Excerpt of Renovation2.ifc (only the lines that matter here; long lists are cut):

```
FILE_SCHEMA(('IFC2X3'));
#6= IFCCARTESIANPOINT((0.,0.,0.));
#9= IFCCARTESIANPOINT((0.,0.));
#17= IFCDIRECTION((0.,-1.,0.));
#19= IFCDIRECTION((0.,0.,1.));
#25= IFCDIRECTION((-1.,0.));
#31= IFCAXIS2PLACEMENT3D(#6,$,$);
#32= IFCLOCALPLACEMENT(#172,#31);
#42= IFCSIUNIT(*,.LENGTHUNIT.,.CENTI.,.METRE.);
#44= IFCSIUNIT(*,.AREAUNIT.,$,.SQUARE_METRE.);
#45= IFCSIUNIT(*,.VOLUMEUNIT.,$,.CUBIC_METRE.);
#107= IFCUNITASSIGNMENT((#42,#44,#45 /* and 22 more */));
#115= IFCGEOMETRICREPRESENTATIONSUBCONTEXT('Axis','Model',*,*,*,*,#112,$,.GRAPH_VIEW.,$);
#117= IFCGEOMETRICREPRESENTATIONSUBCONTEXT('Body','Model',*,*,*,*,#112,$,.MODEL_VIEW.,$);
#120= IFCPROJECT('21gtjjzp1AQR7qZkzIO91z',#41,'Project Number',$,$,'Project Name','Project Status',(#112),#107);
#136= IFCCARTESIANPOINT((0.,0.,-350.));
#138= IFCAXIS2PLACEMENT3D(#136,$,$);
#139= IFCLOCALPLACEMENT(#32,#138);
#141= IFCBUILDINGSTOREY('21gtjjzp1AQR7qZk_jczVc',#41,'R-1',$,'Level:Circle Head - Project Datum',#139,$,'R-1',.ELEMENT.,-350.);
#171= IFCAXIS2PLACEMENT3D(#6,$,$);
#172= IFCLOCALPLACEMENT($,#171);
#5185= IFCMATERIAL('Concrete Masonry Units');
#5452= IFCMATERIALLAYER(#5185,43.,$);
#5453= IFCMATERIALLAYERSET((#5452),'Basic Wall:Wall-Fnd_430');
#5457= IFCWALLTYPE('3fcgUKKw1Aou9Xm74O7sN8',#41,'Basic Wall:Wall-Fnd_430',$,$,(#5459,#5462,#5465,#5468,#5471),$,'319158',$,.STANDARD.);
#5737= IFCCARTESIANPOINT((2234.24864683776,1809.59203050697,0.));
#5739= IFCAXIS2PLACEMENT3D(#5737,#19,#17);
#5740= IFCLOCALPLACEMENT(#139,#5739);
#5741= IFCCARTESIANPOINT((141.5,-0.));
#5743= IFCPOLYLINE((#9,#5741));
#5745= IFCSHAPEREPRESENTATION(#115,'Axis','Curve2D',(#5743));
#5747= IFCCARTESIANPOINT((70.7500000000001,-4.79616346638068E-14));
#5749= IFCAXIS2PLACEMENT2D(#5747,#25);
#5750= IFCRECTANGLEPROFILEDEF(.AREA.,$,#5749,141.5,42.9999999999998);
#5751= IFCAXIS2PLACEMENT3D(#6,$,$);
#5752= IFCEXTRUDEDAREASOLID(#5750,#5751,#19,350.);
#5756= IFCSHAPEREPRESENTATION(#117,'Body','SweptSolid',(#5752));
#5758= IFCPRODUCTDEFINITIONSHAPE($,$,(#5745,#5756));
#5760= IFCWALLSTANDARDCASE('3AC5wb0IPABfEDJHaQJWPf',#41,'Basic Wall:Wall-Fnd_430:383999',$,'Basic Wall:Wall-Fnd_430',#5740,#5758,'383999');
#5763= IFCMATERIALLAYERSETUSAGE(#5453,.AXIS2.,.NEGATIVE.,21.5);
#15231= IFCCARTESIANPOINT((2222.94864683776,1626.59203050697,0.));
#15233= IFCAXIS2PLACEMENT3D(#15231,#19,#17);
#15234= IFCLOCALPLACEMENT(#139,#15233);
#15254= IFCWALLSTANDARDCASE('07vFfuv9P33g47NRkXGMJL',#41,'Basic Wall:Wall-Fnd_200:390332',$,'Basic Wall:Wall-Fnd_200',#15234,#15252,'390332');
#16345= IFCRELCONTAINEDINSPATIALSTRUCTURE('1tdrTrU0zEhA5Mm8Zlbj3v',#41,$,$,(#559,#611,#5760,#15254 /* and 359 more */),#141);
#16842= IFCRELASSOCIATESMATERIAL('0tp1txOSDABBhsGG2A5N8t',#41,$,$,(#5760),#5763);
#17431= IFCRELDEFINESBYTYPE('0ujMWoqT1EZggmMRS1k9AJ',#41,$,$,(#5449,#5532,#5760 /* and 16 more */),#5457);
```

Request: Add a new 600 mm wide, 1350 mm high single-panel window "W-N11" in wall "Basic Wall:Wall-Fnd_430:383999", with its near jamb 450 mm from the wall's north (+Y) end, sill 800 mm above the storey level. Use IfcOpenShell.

```python
import numpy as np
import ifcopenshell
import ifcopenshell.api.feature
import ifcopenshell.api.geometry
import ifcopenshell.api.root
import ifcopenshell.api.spatial
import ifcopenshell.api.type
import ifcopenshell.geom
import ifcopenshell.util.element
import ifcopenshell.util.placement
import ifcopenshell.util.representation
import ifcopenshell.util.shape
import ifcopenshell.util.unit

model = ifcopenshell.open("Renovation2.ifc")
unit_scale = ifcopenshell.util.unit.calculate_unit_scale(model)
settings = ifcopenshell.geom.settings()


def volume(element):
    """Net volume in cubic metres, openings subtracted."""
    shape = ifcopenshell.geom.create_shape(settings, element)
    return ifcopenshell.util.shape.get_volume(shape.geometry)


wall = model.by_guid("3AC5wb0IPABfEDJHaQJWPf")
storey = ifcopenshell.util.element.get_container(wall, ifc_class="IfcBuildingStorey")
context = ifcopenshell.util.representation.get_context(model, "Model", "Body", "MODEL_VIEW")
before = volume(wall)

width, height, from_end, sill = 0.6, 1.35, 0.45, 0.8  # metres

# The wall runs along its own X axis, and the end named is its -X end.
wall_shape = ifcopenshell.geom.create_shape(settings, wall)
x, y, z = ifcopenshell.util.shape.get_vertices(wall_shape.geometry).T
start = x.min() + from_end
face, thickness = float(y.min()), float(y.max() - y.min())
wall_matrix = ifcopenshell.util.placement.get_local_placement(wall.ObjectPlacement)
level = ifcopenshell.util.placement.get_local_placement(storey.ObjectPlacement)[2, 3]


def in_wall(x, y):
    """Placement at x, y metres in the wall's axes, at sill height."""
    matrix = wall_matrix.copy()
    matrix[:, 3] = wall_matrix @ np.array([x / unit_scale, y / unit_scale, 0.0, 1.0])
    matrix[2, 3] = level + sill / unit_scale
    return matrix


# Opening: a box that overshoots both wall faces by 50 mm.
opening = ifcopenshell.api.root.create_entity(model, ifc_class="IfcOpeningElement")
box = ifcopenshell.api.geometry.add_wall_representation(
    model, context=context, length=width, height=height, thickness=thickness + 0.1
)
ifcopenshell.api.geometry.assign_representation(model, product=opening, representation=box)
ifcopenshell.api.geometry.edit_object_placement(model, product=opening, matrix=in_wall(start, face - 0.05), is_si=False)
ifcopenshell.api.feature.add_feature(model, feature=opening, element=wall)

window = ifcopenshell.api.root.create_entity(model, ifc_class="IfcWindow", name="W-N11")
window.OverallWidth, window.OverallHeight = width / unit_scale, height / unit_scale
body = ifcopenshell.api.geometry.add_window_representation(
    model,
    context=context,
    overall_width=window.OverallWidth,
    overall_height=window.OverallHeight,
    partition_type="SINGLE_PANEL",
)
ifcopenshell.api.geometry.assign_representation(model, product=window, representation=body)
ifcopenshell.api.spatial.assign_container(model, products=[window], relating_structure=storey)
fills = ifcopenshell.api.feature.add_filling(model, opening=opening, element=window)
fills.OwnerHistory = window.OwnerHistory  # required in IFC2X3

# IFC2X3 keeps the operation on the window style.
style = ifcopenshell.api.root.create_entity(model, ifc_class="IfcWindowStyle", name="W-N11")
style.OperationType, style.ConstructionType = "SINGLE_PANEL", "NOTDEFINED"
style.ParameterTakesPrecedence = style.Sizeable = False
ifcopenshell.api.type.assign_type(model, related_objects=[window], relating_type=style)

# Centre the window in the wall's thickness.
ifcopenshell.api.geometry.edit_object_placement(model, product=window, matrix=in_wall(start, face), is_si=False)
window_shape = ifcopenshell.geom.create_shape(settings, window)
depth = ifcopenshell.util.shape.get_vertices(window_shape.geometry)[:, 1]
offset = face + thickness / 2 - (depth.min() + depth.max()) / 2
ifcopenshell.api.geometry.edit_object_placement(model, product=window, matrix=in_wall(start, offset), is_si=False)

after = volume(wall)

print(f"wall volume {before:.3f} -> {after:.3f} m3")

model.write("Renovation2_edited.ifc")
```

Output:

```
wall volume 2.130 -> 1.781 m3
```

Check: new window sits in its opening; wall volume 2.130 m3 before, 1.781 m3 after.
